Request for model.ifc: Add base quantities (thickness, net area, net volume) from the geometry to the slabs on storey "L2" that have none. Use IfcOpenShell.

First a look at what the model holds.

```python
import ifcopenshell
import ifcopenshell.util.element
import ifcopenshell.util.unit

model = ifcopenshell.open("model.ifc")
print(model.schema)
for unit_type in ("LENGTHUNIT", "AREAUNIT", "VOLUMEUNIT"):
    print(unit_type, ifcopenshell.util.unit.calculate_unit_scale(model, unit_type))
storey = next(s for s in model.by_type("IfcBuildingStorey") if s.Name == "L2")
slabs = [e for e in ifcopenshell.util.element.get_decomposition(storey) if e.is_a("IfcSlab")]
for e in sorted(slabs, key=lambda e: e.id()):
    print(e.id(), e.is_a(), e.Name, list(ifcopenshell.util.element.get_psets(e, qtos_only=True)), sep=" | ")
```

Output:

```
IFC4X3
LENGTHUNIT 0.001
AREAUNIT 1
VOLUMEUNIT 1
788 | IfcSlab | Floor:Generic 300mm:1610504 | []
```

```python
import ifcopenshell
import ifcopenshell.api.pset
import ifcopenshell.geom
import ifcopenshell.util.element
import ifcopenshell.util.shape
import ifcopenshell.util.unit

model = ifcopenshell.open("model.ifc")
unit_scale = ifcopenshell.util.unit.calculate_unit_scale(model)
area_scale = ifcopenshell.util.unit.calculate_unit_scale(model, "AREAUNIT")
volume_scale = ifcopenshell.util.unit.calculate_unit_scale(model, "VOLUMEUNIT")
settings = ifcopenshell.geom.settings()

storey = next(s for s in model.by_type("IfcBuildingStorey") if s.Name == "L2")
slabs = [e for e in ifcopenshell.util.element.get_decomposition(storey) if e.is_a("IfcSlab")]

for e in sorted(slabs, key=lambda e: e.id()):
    if ifcopenshell.util.element.get_psets(e, qtos_only=True, should_inherit=False):
        continue
    # Geometry comes back in metres, in the element's own axes.
    shape = ifcopenshell.geom.create_shape(settings, e)
    values = {
        "Width": ifcopenshell.util.shape.get_z(shape.geometry) / unit_scale,
        "NetArea": ifcopenshell.util.shape.get_footprint_area(shape.geometry) / area_scale,
        "NetVolume": ifcopenshell.util.shape.get_volume(shape.geometry) / volume_scale,
    }
    qto = ifcopenshell.api.pset.add_qto(model, product=e, name="Qto_SlabBaseQuantities")
    ifcopenshell.api.pset.edit_qto(model, qto=qto, properties=values)
    print(e.id(), {k: round(v, 3) for k, v in values.items()})

model.write("model_v2.ifc")
```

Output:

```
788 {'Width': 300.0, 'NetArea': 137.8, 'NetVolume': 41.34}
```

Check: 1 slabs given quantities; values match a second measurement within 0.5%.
